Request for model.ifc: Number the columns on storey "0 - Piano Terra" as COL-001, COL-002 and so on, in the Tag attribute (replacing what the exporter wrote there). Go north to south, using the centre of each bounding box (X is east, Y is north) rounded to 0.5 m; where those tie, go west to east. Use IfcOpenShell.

First a look at what the model holds.

```python
import ifcopenshell
import ifcopenshell.util.element
import ifcopenshell.util.placement

model = ifcopenshell.open("model.ifc")
print(model.schema)
storey = next(s for s in model.by_type("IfcBuildingStorey") if s.Name == "0 - Piano Terra")
columns = [e for e in ifcopenshell.util.element.get_decomposition(storey) if e.is_a("IfcColumn")]
for e in sorted(columns, key=lambda e: e.id()):
    origin = ifcopenshell.util.placement.get_local_placement(e.ObjectPlacement)[:3, 3]
    print(e.id(), e.Tag, e.Name, origin.round(2) + 0.0, sep=" | ")
```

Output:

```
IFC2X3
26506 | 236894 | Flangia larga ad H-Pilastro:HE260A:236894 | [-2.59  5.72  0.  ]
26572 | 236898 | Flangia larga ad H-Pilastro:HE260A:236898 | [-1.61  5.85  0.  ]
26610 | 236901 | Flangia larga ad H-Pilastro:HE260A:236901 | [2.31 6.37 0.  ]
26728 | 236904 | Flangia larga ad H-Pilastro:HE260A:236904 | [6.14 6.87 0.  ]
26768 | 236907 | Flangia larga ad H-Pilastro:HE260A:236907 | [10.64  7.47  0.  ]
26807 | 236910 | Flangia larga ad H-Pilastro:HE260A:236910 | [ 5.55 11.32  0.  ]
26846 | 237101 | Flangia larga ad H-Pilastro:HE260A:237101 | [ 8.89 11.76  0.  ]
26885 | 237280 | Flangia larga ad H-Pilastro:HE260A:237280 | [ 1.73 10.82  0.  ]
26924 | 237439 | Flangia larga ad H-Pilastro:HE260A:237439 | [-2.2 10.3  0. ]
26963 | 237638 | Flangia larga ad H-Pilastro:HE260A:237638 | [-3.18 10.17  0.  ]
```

```python
import ifcopenshell
import ifcopenshell.geom
import ifcopenshell.util.element
import ifcopenshell.util.shape

model = ifcopenshell.open("model.ifc")
settings = ifcopenshell.geom.settings()
settings.set("use-world-coords", True)


def centre(element):
    shape = ifcopenshell.geom.create_shape(settings, element)
    return ifcopenshell.util.shape.get_bbox_centroid(shape.geometry)


storey = next(s for s in model.by_type("IfcBuildingStorey") if s.Name == "0 - Piano Terra")
columns = [e for e in ifcopenshell.util.element.get_decomposition(storey) if e.is_a("IfcColumn")]

# Insertion points can sit at a corner or the storey origin, so sort by the geometry (in metres).
centres = {e: centre(e) for e in columns}
columns.sort(key=lambda e: (-round(centres[e][1] / 0.5), centres[e][0]))

for i, e in enumerate(columns, start=1):
    number = f"COL-0{i:02d}"
    e.Tag = number
    print(e.id(), number)

model.write("model_rev.ifc")
```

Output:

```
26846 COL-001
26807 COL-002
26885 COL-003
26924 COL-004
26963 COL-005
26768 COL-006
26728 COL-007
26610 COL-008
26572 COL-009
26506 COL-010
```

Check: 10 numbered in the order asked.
